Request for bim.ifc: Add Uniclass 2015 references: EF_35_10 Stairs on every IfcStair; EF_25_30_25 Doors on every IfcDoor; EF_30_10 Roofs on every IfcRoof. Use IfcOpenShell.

First a look at what the model holds.

```python
import ifcopenshell

model = ifcopenshell.open("bim.ifc")
print(model.schema)
print("classifications:", [c.Name for c in model.by_type("IfcClassification")])
for ifc_class in ("IfcDoor", "IfcRoof", "IfcStair", "IfcWall", "IfcWindow"):
    print(ifc_class, len(model.by_type(ifc_class)))
```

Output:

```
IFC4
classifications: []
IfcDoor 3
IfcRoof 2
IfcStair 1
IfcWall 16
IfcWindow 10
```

```python
import ifcopenshell
import ifcopenshell.api.classification

model = ifcopenshell.open("bim.ifc")

system = ifcopenshell.api.classification.add_classification(model, classification="Uniclass 2015")

codes = {
    "IfcStair": ("EF_35_10", "Stairs"),
    "IfcDoor": ("EF_25_30_25", "Doors"),
    "IfcRoof": ("EF_30_10", "Roofs"),
}
for ifc_class, (code, name) in codes.items():
    products = model.by_type(ifc_class)
    ifcopenshell.api.classification.add_reference(
        model, products=products, classification=system, identification=code, name=name
    )
    print(code, len(products))

model.write("bim_updated.ifc")
```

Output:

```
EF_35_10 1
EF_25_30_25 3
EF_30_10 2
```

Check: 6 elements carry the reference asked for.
